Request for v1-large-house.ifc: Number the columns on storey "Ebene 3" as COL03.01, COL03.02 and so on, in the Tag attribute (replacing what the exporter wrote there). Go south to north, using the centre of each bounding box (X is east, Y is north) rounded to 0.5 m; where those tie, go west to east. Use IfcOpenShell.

First a look at what the model holds.

```python
import ifcopenshell
import ifcopenshell.util.element
import ifcopenshell.util.placement

model = ifcopenshell.open("v1-large-house.ifc")
print(model.schema)
storey = next(s for s in model.by_type("IfcBuildingStorey") if s.Name == "Ebene 3")
columns = [e for e in ifcopenshell.util.element.get_decomposition(storey) if e.is_a("IfcColumn")]
for e in sorted(columns, key=lambda e: e.id()):
    origin = ifcopenshell.util.placement.get_local_placement(e.ObjectPlacement)[:3, 3]
    print(e.id(), e.Tag, e.Name, origin.round(2) + 0.0, sep=" | ")
```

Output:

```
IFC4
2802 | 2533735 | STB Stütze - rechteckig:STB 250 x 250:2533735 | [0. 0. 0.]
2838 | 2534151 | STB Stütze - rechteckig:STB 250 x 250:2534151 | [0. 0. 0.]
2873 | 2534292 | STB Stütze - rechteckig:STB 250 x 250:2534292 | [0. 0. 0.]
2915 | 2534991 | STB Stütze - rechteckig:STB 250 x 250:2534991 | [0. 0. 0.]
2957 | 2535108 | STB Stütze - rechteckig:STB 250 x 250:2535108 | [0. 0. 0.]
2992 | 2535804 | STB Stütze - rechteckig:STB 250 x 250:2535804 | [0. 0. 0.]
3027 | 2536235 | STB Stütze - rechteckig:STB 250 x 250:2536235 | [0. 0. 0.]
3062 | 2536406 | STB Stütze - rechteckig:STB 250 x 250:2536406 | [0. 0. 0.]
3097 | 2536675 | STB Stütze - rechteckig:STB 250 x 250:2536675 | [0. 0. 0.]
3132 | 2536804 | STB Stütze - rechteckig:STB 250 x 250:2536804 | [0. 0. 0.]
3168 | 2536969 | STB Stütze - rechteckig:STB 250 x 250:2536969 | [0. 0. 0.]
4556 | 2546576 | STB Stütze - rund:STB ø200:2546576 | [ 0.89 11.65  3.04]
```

```python
import ifcopenshell
import ifcopenshell.geom
import ifcopenshell.util.element
import ifcopenshell.util.shape

model = ifcopenshell.open("v1-large-house.ifc")
settings = ifcopenshell.geom.settings()
settings.set("use-world-coords", True)


def centre(element):
    shape = ifcopenshell.geom.create_shape(settings, element)
    return ifcopenshell.util.shape.get_bbox_centroid(shape.geometry)


storey = next(s for s in model.by_type("IfcBuildingStorey") if s.Name == "Ebene 3")
columns = [e for e in ifcopenshell.util.element.get_decomposition(storey) if e.is_a("IfcColumn")]

# Insertion points can sit at a corner or the storey origin, so sort by the geometry (in metres).
centres = {e: centre(e) for e in columns}
columns.sort(key=lambda e: (round(centres[e][1] / 0.5), centres[e][0]))

for i, e in enumerate(columns, start=1):
    number = f"COL03.{i:02d}"
    e.Tag = number
    print(e.id(), number)

model.write("v1-large-house_v2.ifc")
```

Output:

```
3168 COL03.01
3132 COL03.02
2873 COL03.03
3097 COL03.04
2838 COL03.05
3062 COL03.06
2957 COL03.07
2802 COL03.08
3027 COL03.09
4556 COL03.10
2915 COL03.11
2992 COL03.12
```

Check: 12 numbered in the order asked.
